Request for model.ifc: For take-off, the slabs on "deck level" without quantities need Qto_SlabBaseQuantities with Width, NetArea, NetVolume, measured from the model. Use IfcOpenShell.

First a look at what the model holds.

```python
import ifcopenshell
import ifcopenshell.util.element
import ifcopenshell.util.unit

model = ifcopenshell.open("model.ifc")
print(model.schema)
for unit_type in ("LENGTHUNIT", "AREAUNIT", "VOLUMEUNIT"):
    print(unit_type, ifcopenshell.util.unit.calculate_unit_scale(model, unit_type))
storey = next(s for s in model.by_type("IfcBuildingStorey") if s.Name == "deck level")
slabs = [e for e in ifcopenshell.util.element.get_decomposition(storey) if e.is_a("IfcSlab")]
for e in sorted(slabs, key=lambda e: e.id()):
    print(e.id(), e.is_a(), e.Name, list(ifcopenshell.util.element.get_psets(e, qtos_only=True)), sep=" | ")
```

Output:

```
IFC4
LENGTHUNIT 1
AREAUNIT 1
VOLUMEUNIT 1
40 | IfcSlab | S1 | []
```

```python
import ifcopenshell
import ifcopenshell.api.pset
import ifcopenshell.geom
import ifcopenshell.util.element
import ifcopenshell.util.shape
import ifcopenshell.util.unit

model = ifcopenshell.open("model.ifc")
unit_scale = ifcopenshell.util.unit.calculate_unit_scale(model)
area_scale = ifcopenshell.util.unit.calculate_unit_scale(model, "AREAUNIT")
volume_scale = ifcopenshell.util.unit.calculate_unit_scale(model, "VOLUMEUNIT")
settings = ifcopenshell.geom.settings()

storey = next(s for s in model.by_type("IfcBuildingStorey") if s.Name == "deck level")
slabs = [e for e in ifcopenshell.util.element.get_decomposition(storey) if e.is_a("IfcSlab")]

for e in sorted(slabs, key=lambda e: e.id()):
    if ifcopenshell.util.element.get_psets(e, qtos_only=True, should_inherit=False):
        continue
    # Geometry comes back in metres, in the element's own axes.
    shape = ifcopenshell.geom.create_shape(settings, e)
    values = {
        "Width": ifcopenshell.util.shape.get_z(shape.geometry) / unit_scale,
        "NetArea": ifcopenshell.util.shape.get_footprint_area(shape.geometry) / area_scale,
        "NetVolume": ifcopenshell.util.shape.get_volume(shape.geometry) / volume_scale,
    }
    qto = ifcopenshell.api.pset.add_qto(model, product=e, name="Qto_SlabBaseQuantities")
    ifcopenshell.api.pset.edit_qto(model, qto=qto, properties=values)
    print(e.id(), {k: round(v, 3) for k, v in values.items()})

model.write("model_rev.ifc")
```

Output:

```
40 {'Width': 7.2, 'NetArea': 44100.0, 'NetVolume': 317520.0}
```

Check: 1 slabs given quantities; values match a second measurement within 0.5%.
